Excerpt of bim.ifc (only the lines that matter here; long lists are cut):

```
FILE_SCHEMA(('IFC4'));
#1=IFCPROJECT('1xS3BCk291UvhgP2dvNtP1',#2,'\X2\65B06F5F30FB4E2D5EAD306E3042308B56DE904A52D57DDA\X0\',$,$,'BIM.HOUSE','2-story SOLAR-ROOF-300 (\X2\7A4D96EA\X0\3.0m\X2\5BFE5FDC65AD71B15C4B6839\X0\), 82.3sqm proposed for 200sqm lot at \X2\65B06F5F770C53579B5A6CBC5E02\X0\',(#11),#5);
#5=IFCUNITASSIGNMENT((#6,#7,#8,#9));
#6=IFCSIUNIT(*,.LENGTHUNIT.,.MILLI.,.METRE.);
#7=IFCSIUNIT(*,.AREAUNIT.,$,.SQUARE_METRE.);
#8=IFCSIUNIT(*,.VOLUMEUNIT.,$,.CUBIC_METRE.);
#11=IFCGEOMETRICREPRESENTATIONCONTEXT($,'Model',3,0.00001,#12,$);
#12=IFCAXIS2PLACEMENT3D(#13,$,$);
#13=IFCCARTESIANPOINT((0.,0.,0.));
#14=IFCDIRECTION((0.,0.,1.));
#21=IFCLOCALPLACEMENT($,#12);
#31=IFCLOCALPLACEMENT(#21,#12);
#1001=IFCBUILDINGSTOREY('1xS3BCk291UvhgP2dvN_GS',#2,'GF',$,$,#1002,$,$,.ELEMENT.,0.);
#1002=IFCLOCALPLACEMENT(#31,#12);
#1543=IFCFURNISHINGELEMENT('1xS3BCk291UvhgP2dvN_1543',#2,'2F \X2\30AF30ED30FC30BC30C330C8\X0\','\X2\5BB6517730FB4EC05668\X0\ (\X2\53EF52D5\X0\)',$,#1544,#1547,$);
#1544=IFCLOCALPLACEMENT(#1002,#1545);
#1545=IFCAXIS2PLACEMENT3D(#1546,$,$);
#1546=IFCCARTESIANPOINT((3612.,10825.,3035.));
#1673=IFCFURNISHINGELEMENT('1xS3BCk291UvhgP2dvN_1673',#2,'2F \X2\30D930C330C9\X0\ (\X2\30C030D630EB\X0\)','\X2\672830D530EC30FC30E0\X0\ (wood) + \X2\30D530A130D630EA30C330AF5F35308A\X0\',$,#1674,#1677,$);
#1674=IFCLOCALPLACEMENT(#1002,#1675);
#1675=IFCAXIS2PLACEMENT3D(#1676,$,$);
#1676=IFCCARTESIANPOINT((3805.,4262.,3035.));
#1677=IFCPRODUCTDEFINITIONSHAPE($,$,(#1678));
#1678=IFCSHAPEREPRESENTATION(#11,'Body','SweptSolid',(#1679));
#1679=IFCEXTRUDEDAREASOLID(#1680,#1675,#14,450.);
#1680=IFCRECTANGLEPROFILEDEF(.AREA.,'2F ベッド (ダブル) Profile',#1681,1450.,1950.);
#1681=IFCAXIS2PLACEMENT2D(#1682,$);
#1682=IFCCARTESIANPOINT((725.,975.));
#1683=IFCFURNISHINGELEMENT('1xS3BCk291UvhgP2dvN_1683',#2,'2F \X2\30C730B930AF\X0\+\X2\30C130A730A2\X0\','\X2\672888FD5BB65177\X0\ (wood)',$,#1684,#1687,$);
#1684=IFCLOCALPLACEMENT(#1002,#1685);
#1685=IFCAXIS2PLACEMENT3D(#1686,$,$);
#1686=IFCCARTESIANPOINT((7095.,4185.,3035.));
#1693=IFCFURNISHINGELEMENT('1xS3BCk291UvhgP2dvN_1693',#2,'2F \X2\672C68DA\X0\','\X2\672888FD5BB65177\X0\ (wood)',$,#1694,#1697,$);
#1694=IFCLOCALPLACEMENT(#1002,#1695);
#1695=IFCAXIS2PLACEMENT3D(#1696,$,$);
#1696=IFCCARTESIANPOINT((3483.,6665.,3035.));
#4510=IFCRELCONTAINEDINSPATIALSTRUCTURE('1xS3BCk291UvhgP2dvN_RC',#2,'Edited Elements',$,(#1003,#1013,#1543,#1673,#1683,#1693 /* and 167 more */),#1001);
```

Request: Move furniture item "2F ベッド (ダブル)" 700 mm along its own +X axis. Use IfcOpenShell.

```python
import ifcopenshell
import ifcopenshell.api.geometry
import ifcopenshell.util.placement

model = ifcopenshell.open("bim.ifc")

item = model.by_id(1673)
matrix = ifcopenshell.util.placement.get_local_placement(item.ObjectPlacement)
matrix[:3, 3] += matrix[:3, 0] * 700.0
ifcopenshell.api.geometry.edit_object_placement(model, product=item, matrix=matrix, is_si=False)

print(ifcopenshell.util.placement.get_local_placement(item.ObjectPlacement).round(3) + 0.0)

model.write("bim_edited.ifc")
```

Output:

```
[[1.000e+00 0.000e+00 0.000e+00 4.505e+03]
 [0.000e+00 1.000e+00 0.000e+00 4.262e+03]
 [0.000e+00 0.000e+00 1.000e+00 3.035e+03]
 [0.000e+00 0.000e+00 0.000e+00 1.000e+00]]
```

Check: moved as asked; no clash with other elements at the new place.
